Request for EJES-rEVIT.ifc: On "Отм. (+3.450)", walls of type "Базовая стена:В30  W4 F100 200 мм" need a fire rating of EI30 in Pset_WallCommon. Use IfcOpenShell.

First a look at what the model holds.

```python
import ifcopenshell
import ifcopenshell.util.element

model = ifcopenshell.open("EJES-rEVIT.ifc")
print(model.schema)
storey = next(s for s in model.by_type("IfcBuildingStorey") if s.Name == "Отм. (+3.450)")
walls = [e for e in ifcopenshell.util.element.get_decomposition(storey) if e.is_a("IfcWall")]
seen = {}
for e in walls:
    element_type = ifcopenshell.util.element.get_type(e)
    key = (element_type.Name if element_type != e and element_type else None, ifcopenshell.util.element.get_pset(e, "Pset_WallCommon", "FireRating"))
    seen[key] = seen.get(key, 0) + 1
for (name, value), count in sorted(seen.items(), key=str):
    print(count, "x", name, "|", value)
```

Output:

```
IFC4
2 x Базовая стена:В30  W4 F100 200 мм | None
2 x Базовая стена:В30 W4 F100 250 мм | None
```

```python
import ifcopenshell
import ifcopenshell.api.pset
import ifcopenshell.util.element

model = ifcopenshell.open("EJES-rEVIT.ifc")

storey = next(s for s in model.by_type("IfcBuildingStorey") if s.Name == "Отм. (+3.450)")
walls = [e for e in ifcopenshell.util.element.get_decomposition(storey) if e.is_a("IfcWall")]

count = 0
for e in walls:
    element_type = ifcopenshell.util.element.get_type(e)
    if element_type in (None, e) or element_type.Name != "Базовая стена:В30  W4 F100 200 мм":
        continue
    # add_pset returns the element's existing set when there is one.
    pset = ifcopenshell.api.pset.add_pset(model, product=e, name="Pset_WallCommon")
    ifcopenshell.api.pset.edit_pset(model, pset=pset, properties={"FireRating": "EI30"})
    count += 1

print(count, "walls updated")

model.write("EJES-rEVIT_edited.ifc")
```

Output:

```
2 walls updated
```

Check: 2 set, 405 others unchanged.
